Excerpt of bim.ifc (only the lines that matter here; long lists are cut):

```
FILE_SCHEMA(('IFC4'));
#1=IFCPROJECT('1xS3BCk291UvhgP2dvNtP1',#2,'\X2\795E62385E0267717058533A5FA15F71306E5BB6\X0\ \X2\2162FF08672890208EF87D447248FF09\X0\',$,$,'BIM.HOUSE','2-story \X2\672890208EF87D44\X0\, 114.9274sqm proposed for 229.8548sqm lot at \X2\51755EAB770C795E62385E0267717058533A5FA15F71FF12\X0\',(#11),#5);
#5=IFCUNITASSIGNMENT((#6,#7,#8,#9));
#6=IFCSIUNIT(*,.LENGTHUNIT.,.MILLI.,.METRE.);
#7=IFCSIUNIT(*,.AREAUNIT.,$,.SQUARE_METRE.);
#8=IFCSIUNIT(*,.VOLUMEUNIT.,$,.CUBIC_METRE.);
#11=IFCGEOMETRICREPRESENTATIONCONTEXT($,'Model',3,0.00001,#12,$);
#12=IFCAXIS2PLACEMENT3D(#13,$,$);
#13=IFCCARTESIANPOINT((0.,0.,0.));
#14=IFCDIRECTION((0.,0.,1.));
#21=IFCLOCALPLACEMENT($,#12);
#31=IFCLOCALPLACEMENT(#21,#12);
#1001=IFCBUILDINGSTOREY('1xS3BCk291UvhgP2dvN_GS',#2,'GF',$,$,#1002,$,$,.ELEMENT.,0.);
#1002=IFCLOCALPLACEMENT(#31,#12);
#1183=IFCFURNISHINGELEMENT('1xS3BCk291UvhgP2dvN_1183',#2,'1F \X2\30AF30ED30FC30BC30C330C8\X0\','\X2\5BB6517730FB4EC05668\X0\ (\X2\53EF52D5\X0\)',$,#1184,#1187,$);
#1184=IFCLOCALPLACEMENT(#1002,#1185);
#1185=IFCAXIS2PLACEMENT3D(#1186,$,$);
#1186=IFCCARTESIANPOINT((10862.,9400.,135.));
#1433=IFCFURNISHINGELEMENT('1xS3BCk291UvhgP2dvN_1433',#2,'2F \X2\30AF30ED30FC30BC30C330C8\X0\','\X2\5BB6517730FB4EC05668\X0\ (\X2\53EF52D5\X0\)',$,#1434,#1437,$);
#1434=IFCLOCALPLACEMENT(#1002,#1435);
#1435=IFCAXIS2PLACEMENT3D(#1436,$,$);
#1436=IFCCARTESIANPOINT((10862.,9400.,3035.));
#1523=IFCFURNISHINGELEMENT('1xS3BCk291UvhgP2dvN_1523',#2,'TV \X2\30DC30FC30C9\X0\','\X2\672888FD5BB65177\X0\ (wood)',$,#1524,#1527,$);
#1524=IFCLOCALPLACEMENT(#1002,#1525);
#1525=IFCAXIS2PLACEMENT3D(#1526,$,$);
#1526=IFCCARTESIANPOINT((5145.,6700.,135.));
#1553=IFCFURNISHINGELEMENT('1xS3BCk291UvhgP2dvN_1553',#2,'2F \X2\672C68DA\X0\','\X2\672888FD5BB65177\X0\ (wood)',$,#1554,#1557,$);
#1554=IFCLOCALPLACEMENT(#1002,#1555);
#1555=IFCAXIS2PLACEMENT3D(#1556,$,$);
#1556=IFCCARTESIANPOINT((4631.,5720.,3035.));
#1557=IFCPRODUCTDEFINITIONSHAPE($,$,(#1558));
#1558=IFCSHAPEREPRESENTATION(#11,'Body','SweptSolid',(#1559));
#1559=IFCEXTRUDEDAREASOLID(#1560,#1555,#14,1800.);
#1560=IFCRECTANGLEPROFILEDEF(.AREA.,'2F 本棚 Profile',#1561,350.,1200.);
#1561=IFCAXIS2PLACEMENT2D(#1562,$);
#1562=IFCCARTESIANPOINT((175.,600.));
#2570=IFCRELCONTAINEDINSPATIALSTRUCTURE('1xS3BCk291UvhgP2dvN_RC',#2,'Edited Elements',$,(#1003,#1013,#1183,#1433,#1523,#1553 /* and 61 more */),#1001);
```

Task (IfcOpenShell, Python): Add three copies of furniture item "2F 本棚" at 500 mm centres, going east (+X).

```python
import numpy as np
import ifcopenshell
import ifcopenshell.api.geometry
import ifcopenshell.api.root
import ifcopenshell.util.element
import ifcopenshell.util.placement
import ifcopenshell.util.unit

model = ifcopenshell.open("bim.ifc")
unit_scale = ifcopenshell.util.unit.calculate_unit_scale(model)


def reuse_history(source, copy):
    """copy_class also copies each property set's owner history, people and application; keep the originals."""
    for rel in copy.IsDefinedBy:
        if rel.is_a("IfcRelDefinesByProperties") and (history := rel.RelatingPropertyDefinition.OwnerHistory):
            rel.RelatingPropertyDefinition.OwnerHistory = source.OwnerHistory
            ifcopenshell.util.element.remove_deep2(model, history)


source = model.by_id(1553)
base = ifcopenshell.util.placement.get_local_placement(source.ObjectPlacement)
step = np.array([1.0, 0.0, 0.0]) * 0.5 / unit_scale

for i in range(1, 4):
    copy = ifcopenshell.api.root.copy_class(model, product=source)
    copy.Representation = ifcopenshell.util.element.copy_deep(
        model, source.Representation, exclude=["IfcGeometricRepresentationContext", "IfcRepresentationMap"]
    )
    reuse_history(source, copy)
    matrix = base.copy()
    matrix[:3, 3] += i * step
    print("added at", matrix[:3, 3].round(3) + 0.0)
    ifcopenshell.api.geometry.edit_object_placement(model, product=copy, matrix=matrix, is_si=False)

model.write("bim_updated.ifc")
```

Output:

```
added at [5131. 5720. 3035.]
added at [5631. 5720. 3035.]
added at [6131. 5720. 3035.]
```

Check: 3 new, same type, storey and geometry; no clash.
